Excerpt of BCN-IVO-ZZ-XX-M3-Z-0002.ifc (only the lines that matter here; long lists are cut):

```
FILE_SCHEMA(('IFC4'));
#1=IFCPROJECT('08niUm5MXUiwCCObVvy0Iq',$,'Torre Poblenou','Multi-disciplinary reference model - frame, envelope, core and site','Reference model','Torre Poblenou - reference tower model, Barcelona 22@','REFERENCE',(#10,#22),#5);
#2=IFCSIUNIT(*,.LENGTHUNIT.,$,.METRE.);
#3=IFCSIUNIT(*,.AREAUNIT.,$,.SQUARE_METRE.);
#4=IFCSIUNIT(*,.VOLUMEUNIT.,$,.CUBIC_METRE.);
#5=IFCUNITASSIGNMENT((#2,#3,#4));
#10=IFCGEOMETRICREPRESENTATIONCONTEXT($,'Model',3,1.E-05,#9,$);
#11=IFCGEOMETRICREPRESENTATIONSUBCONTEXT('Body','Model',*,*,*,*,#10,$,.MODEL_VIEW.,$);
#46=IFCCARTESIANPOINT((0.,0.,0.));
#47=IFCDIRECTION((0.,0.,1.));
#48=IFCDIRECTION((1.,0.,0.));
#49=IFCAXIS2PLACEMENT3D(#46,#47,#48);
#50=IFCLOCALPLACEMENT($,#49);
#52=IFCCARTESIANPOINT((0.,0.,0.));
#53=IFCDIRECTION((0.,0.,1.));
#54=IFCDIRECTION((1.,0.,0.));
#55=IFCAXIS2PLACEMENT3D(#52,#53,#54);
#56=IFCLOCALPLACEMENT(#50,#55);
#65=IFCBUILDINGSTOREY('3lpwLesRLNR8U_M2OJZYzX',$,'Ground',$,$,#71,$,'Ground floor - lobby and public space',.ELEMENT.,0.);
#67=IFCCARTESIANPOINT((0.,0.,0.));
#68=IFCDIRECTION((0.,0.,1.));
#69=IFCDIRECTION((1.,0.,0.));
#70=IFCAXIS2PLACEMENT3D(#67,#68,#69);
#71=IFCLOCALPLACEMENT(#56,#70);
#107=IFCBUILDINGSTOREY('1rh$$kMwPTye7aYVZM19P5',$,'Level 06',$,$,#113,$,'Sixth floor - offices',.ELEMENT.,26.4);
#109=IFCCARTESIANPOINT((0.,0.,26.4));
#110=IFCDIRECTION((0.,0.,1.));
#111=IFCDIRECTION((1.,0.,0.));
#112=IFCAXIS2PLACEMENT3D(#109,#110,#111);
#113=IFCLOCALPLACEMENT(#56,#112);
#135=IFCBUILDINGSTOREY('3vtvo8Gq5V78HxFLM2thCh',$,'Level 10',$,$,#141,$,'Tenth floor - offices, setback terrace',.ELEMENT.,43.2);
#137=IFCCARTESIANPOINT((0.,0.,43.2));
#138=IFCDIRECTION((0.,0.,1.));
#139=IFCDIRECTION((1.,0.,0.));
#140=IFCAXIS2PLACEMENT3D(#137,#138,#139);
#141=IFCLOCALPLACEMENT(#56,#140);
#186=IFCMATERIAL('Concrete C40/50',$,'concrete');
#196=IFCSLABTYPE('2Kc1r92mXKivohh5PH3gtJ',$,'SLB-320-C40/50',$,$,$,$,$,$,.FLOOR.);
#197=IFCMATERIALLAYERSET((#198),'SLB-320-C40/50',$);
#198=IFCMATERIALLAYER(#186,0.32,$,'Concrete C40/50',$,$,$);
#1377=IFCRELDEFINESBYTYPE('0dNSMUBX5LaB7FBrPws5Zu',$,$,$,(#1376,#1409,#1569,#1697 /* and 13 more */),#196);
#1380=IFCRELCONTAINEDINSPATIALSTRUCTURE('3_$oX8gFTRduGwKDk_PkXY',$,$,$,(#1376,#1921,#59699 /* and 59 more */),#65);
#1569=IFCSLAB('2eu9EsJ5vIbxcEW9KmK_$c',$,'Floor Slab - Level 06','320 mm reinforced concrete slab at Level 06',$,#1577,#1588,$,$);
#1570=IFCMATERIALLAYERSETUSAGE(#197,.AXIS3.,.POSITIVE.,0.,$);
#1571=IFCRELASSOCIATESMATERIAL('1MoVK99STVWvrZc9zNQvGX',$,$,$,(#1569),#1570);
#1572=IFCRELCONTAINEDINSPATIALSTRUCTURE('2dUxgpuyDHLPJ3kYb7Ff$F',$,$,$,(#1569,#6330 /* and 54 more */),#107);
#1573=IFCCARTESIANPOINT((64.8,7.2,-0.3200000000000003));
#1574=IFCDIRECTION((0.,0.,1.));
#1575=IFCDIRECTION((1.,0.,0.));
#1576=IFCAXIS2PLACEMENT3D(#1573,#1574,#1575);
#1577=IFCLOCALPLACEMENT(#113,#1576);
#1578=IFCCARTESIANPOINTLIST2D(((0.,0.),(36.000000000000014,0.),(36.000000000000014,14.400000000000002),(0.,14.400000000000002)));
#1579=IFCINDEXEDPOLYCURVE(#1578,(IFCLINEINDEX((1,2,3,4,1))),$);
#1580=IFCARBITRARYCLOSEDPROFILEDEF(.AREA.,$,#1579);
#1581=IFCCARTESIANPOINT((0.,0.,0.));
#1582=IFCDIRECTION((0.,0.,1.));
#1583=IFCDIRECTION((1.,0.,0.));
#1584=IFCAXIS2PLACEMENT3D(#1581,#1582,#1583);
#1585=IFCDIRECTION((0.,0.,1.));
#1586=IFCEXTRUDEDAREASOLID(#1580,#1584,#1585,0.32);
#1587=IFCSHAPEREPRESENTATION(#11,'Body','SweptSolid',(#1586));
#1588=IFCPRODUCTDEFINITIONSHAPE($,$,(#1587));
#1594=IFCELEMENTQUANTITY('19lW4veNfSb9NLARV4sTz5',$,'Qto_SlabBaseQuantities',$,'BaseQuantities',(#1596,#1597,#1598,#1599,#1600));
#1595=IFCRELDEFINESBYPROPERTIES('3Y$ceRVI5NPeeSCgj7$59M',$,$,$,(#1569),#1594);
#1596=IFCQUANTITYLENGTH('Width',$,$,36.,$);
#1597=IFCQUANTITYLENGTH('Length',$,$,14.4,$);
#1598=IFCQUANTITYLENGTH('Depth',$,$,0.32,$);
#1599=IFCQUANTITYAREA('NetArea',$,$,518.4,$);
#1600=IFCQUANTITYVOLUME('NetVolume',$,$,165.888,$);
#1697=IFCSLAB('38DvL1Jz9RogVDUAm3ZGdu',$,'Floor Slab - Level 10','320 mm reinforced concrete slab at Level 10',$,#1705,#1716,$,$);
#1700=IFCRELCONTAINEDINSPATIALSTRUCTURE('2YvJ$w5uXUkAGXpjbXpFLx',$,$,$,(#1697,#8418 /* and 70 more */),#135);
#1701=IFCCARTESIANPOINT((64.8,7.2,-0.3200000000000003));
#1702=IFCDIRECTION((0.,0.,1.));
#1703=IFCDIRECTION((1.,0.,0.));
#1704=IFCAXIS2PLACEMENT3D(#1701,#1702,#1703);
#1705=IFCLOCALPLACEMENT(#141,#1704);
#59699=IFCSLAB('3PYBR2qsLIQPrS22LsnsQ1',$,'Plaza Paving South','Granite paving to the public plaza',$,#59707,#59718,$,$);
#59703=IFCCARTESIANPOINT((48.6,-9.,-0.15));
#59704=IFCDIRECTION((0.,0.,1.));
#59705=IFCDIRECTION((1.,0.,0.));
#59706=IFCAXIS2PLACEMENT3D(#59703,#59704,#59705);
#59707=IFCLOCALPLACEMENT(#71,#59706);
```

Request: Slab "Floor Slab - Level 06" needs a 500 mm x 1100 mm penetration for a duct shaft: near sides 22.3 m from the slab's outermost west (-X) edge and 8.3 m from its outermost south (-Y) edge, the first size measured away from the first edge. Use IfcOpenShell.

```python
import numpy as np
import ifcopenshell
import ifcopenshell.api.feature
import ifcopenshell.api.geometry
import ifcopenshell.api.pset
import ifcopenshell.api.root
import ifcopenshell.geom
import ifcopenshell.util.element
import ifcopenshell.util.placement
import ifcopenshell.util.representation
import ifcopenshell.util.shape
import ifcopenshell.util.unit

model = ifcopenshell.open("BCN-IVO-ZZ-XX-M3-Z-0002.ifc")
unit_scale = ifcopenshell.util.unit.calculate_unit_scale(model)
area_scale = ifcopenshell.util.unit.calculate_unit_scale(model, "AREAUNIT")
volume_scale = ifcopenshell.util.unit.calculate_unit_scale(model, "VOLUMEUNIT")
settings = ifcopenshell.geom.settings()


def volume(element):
    """Net volume in cubic metres, openings subtracted."""
    shape = ifcopenshell.geom.create_shape(settings, element)
    return ifcopenshell.util.shape.get_volume(shape.geometry)


slab = model.by_guid("2eu9EsJ5vIbxcEW9KmK_$c")
before = volume(slab)

# Extent in the slab's own axes, in metres. The edges named are its -X and -Y sides.
slab_shape = ifcopenshell.geom.create_shape(settings, slab)
vertices = ifcopenshell.util.shape.get_vertices(slab_shape.geometry)
x_min, y_min, bottom = vertices.min(axis=0)
top = vertices[:, 2].max()

opening = ifcopenshell.api.root.create_entity(model, ifc_class="IfcOpeningElement", name="Duct shaft opening", predefined_type="OPENING")
context = ifcopenshell.util.representation.get_context(model, "Model", "Body", "MODEL_VIEW")
width, depth = 0.5, 1.1
outline = [(0.0, 0.0), (width, 0.0), (width, depth), (0.0, depth), (0.0, 0.0)]
# Overshoot both faces by 50 mm so the cut is clean.
shape = ifcopenshell.api.geometry.add_slab_representation(
    model, context=context, depth=top - bottom + 0.1, polyline=outline
)
ifcopenshell.api.geometry.assign_representation(model, product=opening, representation=shape)

matrix = ifcopenshell.util.placement.get_local_placement(slab.ObjectPlacement)
matrix[:, 3] = matrix @ np.append(np.array([x_min + 22.3, y_min + 8.3, bottom - 0.05]) / unit_scale, 1.0)
ifcopenshell.api.geometry.edit_object_placement(model, product=opening, matrix=matrix, is_si=False)
ifcopenshell.api.feature.add_feature(model, feature=opening, element=slab)

after = volume(slab)

# Update the slab's stored quantities.
qto = model.by_id(ifcopenshell.util.element.get_pset(slab, "Qto_SlabBaseQuantities", should_inherit=False)["id"])
ifcopenshell.api.pset.edit_qto(model, qto=qto, properties={
    "NetArea": after / (top - bottom) / area_scale,
    "NetVolume": after / volume_scale,
})

print(f"slab volume {before:.3f} -> {after:.3f} m3")

model.write("BCN-IVO-ZZ-XX-M3-Z-0002_rev.ifc")
```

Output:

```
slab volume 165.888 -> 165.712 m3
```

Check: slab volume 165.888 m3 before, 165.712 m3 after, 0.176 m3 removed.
